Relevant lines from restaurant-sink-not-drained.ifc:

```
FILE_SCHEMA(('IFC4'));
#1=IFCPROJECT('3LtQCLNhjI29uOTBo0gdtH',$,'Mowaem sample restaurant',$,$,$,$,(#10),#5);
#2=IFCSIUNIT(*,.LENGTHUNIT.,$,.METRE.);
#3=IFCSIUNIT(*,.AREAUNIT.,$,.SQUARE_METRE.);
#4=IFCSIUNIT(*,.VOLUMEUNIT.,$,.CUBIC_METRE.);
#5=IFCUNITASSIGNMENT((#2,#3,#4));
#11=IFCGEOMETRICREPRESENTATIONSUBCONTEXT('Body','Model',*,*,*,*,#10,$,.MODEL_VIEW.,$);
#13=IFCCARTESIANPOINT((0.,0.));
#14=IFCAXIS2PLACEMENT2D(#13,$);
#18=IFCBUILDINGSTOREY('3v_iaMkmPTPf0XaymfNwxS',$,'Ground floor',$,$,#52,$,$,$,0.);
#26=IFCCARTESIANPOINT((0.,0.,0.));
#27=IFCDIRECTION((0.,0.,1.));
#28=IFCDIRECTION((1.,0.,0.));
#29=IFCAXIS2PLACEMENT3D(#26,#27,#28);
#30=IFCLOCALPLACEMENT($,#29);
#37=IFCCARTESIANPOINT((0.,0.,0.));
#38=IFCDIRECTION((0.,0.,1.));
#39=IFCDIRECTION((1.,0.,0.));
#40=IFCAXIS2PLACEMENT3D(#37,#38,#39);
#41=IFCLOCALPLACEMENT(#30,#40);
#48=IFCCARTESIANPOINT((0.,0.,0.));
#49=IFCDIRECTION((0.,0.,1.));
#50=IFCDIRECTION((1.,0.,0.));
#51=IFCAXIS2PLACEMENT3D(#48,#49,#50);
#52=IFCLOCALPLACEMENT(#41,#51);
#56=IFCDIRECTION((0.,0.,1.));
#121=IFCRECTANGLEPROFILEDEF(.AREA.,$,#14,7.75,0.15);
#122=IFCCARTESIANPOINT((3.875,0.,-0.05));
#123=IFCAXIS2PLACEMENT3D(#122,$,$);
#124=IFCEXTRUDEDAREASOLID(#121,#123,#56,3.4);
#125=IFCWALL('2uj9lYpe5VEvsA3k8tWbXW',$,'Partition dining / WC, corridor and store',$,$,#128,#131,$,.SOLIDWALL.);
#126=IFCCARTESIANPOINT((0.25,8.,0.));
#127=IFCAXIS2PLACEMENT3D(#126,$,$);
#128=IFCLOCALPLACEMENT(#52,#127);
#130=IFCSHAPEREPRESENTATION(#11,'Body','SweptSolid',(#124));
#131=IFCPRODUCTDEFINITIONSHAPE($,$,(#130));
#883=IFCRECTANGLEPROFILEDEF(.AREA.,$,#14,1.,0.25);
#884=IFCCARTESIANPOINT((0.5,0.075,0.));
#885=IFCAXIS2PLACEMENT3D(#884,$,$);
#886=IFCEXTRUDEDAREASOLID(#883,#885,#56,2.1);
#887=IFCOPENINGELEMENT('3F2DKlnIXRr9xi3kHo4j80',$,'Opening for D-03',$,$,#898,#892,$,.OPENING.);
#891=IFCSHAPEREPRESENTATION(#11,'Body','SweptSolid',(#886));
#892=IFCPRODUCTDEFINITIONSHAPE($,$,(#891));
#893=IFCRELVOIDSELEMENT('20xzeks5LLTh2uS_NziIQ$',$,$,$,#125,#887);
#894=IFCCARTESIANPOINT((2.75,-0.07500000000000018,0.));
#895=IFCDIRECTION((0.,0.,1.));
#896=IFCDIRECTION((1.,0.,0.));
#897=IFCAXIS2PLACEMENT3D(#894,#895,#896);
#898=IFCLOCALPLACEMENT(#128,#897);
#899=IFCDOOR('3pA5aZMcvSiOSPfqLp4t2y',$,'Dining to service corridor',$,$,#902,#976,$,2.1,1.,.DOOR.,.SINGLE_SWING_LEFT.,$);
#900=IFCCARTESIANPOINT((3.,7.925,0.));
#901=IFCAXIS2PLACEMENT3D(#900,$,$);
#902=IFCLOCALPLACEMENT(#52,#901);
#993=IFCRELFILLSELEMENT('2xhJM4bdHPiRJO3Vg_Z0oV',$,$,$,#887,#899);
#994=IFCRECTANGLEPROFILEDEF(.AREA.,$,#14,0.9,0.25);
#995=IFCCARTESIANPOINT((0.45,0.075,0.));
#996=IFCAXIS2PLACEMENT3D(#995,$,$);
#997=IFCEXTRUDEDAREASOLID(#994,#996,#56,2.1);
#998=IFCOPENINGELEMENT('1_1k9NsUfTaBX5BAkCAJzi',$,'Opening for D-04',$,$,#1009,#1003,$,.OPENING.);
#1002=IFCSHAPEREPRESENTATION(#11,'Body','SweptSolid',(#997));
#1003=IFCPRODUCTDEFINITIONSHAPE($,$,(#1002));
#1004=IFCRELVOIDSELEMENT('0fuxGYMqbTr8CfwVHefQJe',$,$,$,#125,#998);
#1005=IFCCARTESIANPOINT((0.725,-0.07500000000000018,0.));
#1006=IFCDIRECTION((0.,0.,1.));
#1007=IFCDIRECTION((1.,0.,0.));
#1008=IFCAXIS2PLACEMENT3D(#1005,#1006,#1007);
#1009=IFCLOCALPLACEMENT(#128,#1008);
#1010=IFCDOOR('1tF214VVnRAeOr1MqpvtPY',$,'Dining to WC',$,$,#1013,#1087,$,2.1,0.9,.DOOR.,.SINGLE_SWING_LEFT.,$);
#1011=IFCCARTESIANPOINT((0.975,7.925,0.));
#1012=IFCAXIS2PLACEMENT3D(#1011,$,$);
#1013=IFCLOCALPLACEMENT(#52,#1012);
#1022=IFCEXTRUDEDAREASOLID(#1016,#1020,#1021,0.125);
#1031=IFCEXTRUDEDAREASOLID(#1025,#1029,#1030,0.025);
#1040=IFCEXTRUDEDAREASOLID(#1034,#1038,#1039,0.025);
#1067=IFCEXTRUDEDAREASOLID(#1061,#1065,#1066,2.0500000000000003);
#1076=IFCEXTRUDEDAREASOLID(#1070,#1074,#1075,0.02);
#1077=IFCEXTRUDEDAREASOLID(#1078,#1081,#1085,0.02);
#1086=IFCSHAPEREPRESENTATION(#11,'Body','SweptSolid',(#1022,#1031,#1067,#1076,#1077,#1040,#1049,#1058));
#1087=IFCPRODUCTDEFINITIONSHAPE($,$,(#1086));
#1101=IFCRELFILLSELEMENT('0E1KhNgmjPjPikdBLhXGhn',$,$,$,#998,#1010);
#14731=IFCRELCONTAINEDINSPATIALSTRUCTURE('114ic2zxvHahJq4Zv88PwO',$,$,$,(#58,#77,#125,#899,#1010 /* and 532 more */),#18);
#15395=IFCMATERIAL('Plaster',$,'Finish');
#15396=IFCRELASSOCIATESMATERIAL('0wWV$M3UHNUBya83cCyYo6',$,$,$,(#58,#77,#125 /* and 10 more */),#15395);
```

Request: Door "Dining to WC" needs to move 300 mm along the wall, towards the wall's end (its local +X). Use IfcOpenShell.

```python
import ifcopenshell
import ifcopenshell.api.geometry
import ifcopenshell.util.placement
import ifcopenshell.util.unit

model = ifcopenshell.open("restaurant-sink-not-drained.ifc")
unit_scale = ifcopenshell.util.unit.calculate_unit_scale(model)

door = model.by_guid("1tF214VVnRAeOr1MqpvtPY")
opening = door.FillsVoids[0].RelatingOpeningElement
wall = opening.VoidsElements[0].RelatingBuildingElement

wall_matrix = ifcopenshell.util.placement.get_local_placement(wall.ObjectPlacement)
shift = wall_matrix[:3, 0] * 0.3 / unit_scale
before = ifcopenshell.util.placement.get_local_placement(door.ObjectPlacement)[:3, 3].copy()

# The door is not placed relative to its opening, so move both.
for product in (opening, door):
    matrix = ifcopenshell.util.placement.get_local_placement(product.ObjectPlacement)
    matrix[:3, 3] += shift
    ifcopenshell.api.geometry.edit_object_placement(model, product=product, matrix=matrix, is_si=False)

after = ifcopenshell.util.placement.get_local_placement(door.ObjectPlacement)[:3, 3]
print("door moved by", (after - before).round(3) + 0.0)

model.write("restaurant-sink-not-drained_updated.ifc")
```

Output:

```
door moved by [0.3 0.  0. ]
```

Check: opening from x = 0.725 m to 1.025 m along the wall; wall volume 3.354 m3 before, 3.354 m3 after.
